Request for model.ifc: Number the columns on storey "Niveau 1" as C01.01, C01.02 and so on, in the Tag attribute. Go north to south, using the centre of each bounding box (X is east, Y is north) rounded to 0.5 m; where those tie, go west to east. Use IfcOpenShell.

First a look at what the model holds.

```python
import ifcopenshell
import ifcopenshell.util.element
import ifcopenshell.util.placement

model = ifcopenshell.open("model.ifc")
print(model.schema)
storey = next(s for s in model.by_type("IfcBuildingStorey") if s.Name == "Niveau 1")
columns = [e for e in ifcopenshell.util.element.get_decomposition(storey) if e.is_a("IfcColumn")]
for e in sorted(columns, key=lambda e: e.id()):
    origin = ifcopenshell.util.placement.get_local_placement(e.ObjectPlacement)[:3, 3]
    print(e.id(), e.Tag, e.Name, origin.round(2) + 0.0, sep=" | ")
```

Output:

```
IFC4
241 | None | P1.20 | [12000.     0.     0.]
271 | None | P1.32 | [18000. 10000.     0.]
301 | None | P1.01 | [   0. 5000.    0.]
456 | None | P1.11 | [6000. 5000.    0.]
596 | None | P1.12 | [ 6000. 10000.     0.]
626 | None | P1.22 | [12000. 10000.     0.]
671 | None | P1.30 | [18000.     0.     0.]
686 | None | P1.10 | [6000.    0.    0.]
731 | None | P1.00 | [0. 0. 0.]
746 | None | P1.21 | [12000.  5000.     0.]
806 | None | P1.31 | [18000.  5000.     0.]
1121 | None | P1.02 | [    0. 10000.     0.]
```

```python
import ifcopenshell
import ifcopenshell.geom
import ifcopenshell.util.element
import ifcopenshell.util.shape

model = ifcopenshell.open("model.ifc")
settings = ifcopenshell.geom.settings()
settings.set("use-world-coords", True)


def centre(element):
    shape = ifcopenshell.geom.create_shape(settings, element)
    return ifcopenshell.util.shape.get_bbox_centroid(shape.geometry)


storey = next(s for s in model.by_type("IfcBuildingStorey") if s.Name == "Niveau 1")
columns = [e for e in ifcopenshell.util.element.get_decomposition(storey) if e.is_a("IfcColumn")]

# Insertion points can sit at a corner or the storey origin, so sort by the geometry (in metres).
centres = {e: centre(e) for e in columns}
columns.sort(key=lambda e: (-round(centres[e][1] / 0.5), centres[e][0]))

for i, e in enumerate(columns, start=1):
    number = f"C01.{i:02d}"
    e.Tag = number
    print(e.id(), number)

model.write("model-out.ifc")
```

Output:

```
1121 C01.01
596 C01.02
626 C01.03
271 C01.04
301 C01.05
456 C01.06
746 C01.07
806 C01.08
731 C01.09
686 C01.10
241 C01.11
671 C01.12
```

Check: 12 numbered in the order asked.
